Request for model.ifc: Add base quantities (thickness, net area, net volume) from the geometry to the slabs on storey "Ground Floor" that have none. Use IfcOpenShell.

First a look at what the model holds.

```python
import ifcopenshell
import ifcopenshell.util.element
import ifcopenshell.util.unit

model = ifcopenshell.open("model.ifc")
print(model.schema)
for unit_type in ("LENGTHUNIT", "AREAUNIT", "VOLUMEUNIT"):
    print(unit_type, ifcopenshell.util.unit.calculate_unit_scale(model, unit_type))
storey = next(s for s in model.by_type("IfcBuildingStorey") if s.Name == "Ground Floor")
slabs = [e for e in ifcopenshell.util.element.get_decomposition(storey) if e.is_a("IfcSlab")]
for e in sorted(slabs, key=lambda e: e.id()):
    print(e.id(), e.is_a(), e.Name, list(ifcopenshell.util.element.get_psets(e, qtos_only=True)), sep=" | ")
```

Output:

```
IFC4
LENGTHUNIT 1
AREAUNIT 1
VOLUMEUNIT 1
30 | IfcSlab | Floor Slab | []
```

```python
import ifcopenshell
import ifcopenshell.api.pset
import ifcopenshell.geom
import ifcopenshell.util.element
import ifcopenshell.util.shape
import ifcopenshell.util.unit

model = ifcopenshell.open("model.ifc")
unit_scale = ifcopenshell.util.unit.calculate_unit_scale(model)
area_scale = ifcopenshell.util.unit.calculate_unit_scale(model, "AREAUNIT")
volume_scale = ifcopenshell.util.unit.calculate_unit_scale(model, "VOLUMEUNIT")
settings = ifcopenshell.geom.settings()

storey = next(s for s in model.by_type("IfcBuildingStorey") if s.Name == "Ground Floor")
slabs = [e for e in ifcopenshell.util.element.get_decomposition(storey) if e.is_a("IfcSlab")]

for e in sorted(slabs, key=lambda e: e.id()):
    if ifcopenshell.util.element.get_psets(e, qtos_only=True, should_inherit=False):
        continue
    # Geometry comes back in metres, in the element's own axes.
    shape = ifcopenshell.geom.create_shape(settings, e)
    values = {
        "Width": ifcopenshell.util.shape.get_z(shape.geometry) / unit_scale,
        "NetArea": ifcopenshell.util.shape.get_footprint_area(shape.geometry) / area_scale,
        "NetVolume": ifcopenshell.util.shape.get_volume(shape.geometry) / volume_scale,
    }
    qto = ifcopenshell.api.pset.add_qto(model, product=e, name="Qto_SlabBaseQuantities")
    ifcopenshell.api.pset.edit_qto(model, qto=qto, properties=values)
    print(e.id(), {k: round(v, 3) for k, v in values.items()})

model.write("model-out.ifc")
```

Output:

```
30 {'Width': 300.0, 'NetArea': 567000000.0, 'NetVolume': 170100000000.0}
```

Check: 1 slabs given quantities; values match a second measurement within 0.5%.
